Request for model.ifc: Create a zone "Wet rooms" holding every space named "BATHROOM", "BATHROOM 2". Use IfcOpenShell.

First a look at what the model holds.

```python
import ifcopenshell

model = ifcopenshell.open("model.ifc")
print(model.schema)
seen = {}
for space in model.by_type("IfcSpace"):
    seen[space.LongName] = seen.get(space.LongName, 0) + 1
for name, count in sorted(seen.items(), key=str):
    print(count, "x", name)
print("zones:", [z.Name for z in model.by_type("IfcZone")][:20])
```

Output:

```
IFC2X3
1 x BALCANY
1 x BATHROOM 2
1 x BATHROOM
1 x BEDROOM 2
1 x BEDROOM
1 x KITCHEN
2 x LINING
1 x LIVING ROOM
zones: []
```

```python
import ifcopenshell
import ifcopenshell.api.group
import ifcopenshell.api.root

model = ifcopenshell.open("model.ifc")

names = {"BATHROOM", "BATHROOM 2"}
spaces = [s for s in model.by_type("IfcSpace") if s.LongName in names]

zone = ifcopenshell.api.root.create_entity(model, ifc_class="IfcZone", name="Wet rooms")
ifcopenshell.api.group.assign_group(model, products=spaces, group=zone)
print(len(spaces), "spaces in", zone.Name)

model.write("model_edited.ifc")
```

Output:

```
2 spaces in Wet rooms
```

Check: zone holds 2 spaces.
